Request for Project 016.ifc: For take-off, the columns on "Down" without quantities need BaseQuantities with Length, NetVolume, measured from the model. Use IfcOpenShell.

First a look at what the model holds.

```python
import ifcopenshell
import ifcopenshell.util.element
import ifcopenshell.util.unit

model = ifcopenshell.open("Project 016.ifc")
print(model.schema)
for unit_type in ("LENGTHUNIT", "AREAUNIT", "VOLUMEUNIT"):
    print(unit_type, ifcopenshell.util.unit.calculate_unit_scale(model, unit_type))
storey = next(s for s in model.by_type("IfcBuildingStorey") if s.Name == "Down")
columns = [e for e in ifcopenshell.util.element.get_decomposition(storey) if e.is_a("IfcColumn")]
for e in sorted(columns, key=lambda e: e.id()):
    print(e.id(), e.is_a(), e.Name, list(ifcopenshell.util.element.get_psets(e, qtos_only=True)), sep=" | ")
```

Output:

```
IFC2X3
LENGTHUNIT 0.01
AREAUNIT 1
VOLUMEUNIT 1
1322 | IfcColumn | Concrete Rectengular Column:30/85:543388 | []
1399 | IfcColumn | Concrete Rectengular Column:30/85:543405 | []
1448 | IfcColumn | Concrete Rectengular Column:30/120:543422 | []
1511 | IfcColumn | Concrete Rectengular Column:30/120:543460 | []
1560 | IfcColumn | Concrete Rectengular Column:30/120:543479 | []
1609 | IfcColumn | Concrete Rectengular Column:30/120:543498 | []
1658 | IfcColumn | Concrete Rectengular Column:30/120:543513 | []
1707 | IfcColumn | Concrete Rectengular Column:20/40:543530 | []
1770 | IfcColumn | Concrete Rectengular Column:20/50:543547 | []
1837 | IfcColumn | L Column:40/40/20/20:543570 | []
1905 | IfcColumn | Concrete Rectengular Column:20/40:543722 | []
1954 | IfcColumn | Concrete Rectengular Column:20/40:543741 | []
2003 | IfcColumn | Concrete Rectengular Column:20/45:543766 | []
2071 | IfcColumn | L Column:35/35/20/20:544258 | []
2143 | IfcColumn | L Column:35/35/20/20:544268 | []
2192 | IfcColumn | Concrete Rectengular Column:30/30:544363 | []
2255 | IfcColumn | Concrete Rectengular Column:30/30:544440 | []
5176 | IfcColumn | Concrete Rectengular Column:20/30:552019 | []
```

```python
import ifcopenshell
import ifcopenshell.api.pset
import ifcopenshell.geom
import ifcopenshell.util.element
import ifcopenshell.util.shape
import ifcopenshell.util.unit

model = ifcopenshell.open("Project 016.ifc")
unit_scale = ifcopenshell.util.unit.calculate_unit_scale(model)
volume_scale = ifcopenshell.util.unit.calculate_unit_scale(model, "VOLUMEUNIT")
settings = ifcopenshell.geom.settings()

storey = next(s for s in model.by_type("IfcBuildingStorey") if s.Name == "Down")
columns = [e for e in ifcopenshell.util.element.get_decomposition(storey) if e.is_a("IfcColumn")]

for e in sorted(columns, key=lambda e: e.id()):
    if ifcopenshell.util.element.get_psets(e, qtos_only=True, should_inherit=False):
        continue
    # Geometry comes back in metres, in the element's own axes.
    shape = ifcopenshell.geom.create_shape(settings, e)
    values = {
        "Length": ifcopenshell.util.shape.get_z(shape.geometry) / unit_scale,
        "NetVolume": ifcopenshell.util.shape.get_volume(shape.geometry) / volume_scale,
    }
    qto = ifcopenshell.api.pset.add_qto(model, product=e, name="BaseQuantities")
    ifcopenshell.api.pset.edit_qto(model, qto=qto, properties=values)
    print(e.id(), {k: round(v, 3) for k, v in values.items()})

model.write("Project 016_rev.ifc")
```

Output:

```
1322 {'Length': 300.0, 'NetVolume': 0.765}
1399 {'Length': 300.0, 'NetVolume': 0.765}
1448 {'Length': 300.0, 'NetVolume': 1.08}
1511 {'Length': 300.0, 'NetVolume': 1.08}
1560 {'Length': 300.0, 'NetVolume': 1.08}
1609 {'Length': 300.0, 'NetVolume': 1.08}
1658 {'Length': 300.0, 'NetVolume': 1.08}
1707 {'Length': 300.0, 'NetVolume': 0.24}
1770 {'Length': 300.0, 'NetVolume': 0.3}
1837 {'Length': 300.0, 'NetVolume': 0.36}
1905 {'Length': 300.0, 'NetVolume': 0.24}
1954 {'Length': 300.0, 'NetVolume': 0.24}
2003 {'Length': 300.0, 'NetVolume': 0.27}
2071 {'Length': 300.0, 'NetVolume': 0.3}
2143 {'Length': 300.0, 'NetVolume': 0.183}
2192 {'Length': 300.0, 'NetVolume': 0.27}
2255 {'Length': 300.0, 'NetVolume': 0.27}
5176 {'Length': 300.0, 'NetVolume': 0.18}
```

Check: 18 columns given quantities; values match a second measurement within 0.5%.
